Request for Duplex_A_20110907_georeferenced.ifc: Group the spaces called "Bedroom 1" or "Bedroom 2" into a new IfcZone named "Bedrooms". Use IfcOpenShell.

First a look at what the model holds.

```python
import ifcopenshell

model = ifcopenshell.open("Duplex_A_20110907_georeferenced.ifc")
print(model.schema)
seen = {}
for space in model.by_type("IfcSpace"):
    seen[space.LongName] = seen.get(space.LongName, 0) + 1
for name, count in sorted(seen.items(), key=str):
    print(count, "x", name)
print("zones:", [z.Name for z in model.by_type("IfcZone")][:20])
```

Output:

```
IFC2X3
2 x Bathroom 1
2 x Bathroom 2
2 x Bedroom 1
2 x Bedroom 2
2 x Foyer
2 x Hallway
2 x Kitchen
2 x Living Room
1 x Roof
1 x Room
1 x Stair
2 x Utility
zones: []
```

```python
import ifcopenshell
import ifcopenshell.api.group
import ifcopenshell.api.root

model = ifcopenshell.open("Duplex_A_20110907_georeferenced.ifc")

names = {"Bedroom 1", "Bedroom 2"}
spaces = [s for s in model.by_type("IfcSpace") if s.LongName in names]

zone = ifcopenshell.api.root.create_entity(model, ifc_class="IfcZone", name="Bedrooms")
ifcopenshell.api.group.assign_group(model, products=spaces, group=zone)
print(len(spaces), "spaces in", zone.Name)

model.write("Duplex_A_20110907_georeferenced_v2.ifc")
```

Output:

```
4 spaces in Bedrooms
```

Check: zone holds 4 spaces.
